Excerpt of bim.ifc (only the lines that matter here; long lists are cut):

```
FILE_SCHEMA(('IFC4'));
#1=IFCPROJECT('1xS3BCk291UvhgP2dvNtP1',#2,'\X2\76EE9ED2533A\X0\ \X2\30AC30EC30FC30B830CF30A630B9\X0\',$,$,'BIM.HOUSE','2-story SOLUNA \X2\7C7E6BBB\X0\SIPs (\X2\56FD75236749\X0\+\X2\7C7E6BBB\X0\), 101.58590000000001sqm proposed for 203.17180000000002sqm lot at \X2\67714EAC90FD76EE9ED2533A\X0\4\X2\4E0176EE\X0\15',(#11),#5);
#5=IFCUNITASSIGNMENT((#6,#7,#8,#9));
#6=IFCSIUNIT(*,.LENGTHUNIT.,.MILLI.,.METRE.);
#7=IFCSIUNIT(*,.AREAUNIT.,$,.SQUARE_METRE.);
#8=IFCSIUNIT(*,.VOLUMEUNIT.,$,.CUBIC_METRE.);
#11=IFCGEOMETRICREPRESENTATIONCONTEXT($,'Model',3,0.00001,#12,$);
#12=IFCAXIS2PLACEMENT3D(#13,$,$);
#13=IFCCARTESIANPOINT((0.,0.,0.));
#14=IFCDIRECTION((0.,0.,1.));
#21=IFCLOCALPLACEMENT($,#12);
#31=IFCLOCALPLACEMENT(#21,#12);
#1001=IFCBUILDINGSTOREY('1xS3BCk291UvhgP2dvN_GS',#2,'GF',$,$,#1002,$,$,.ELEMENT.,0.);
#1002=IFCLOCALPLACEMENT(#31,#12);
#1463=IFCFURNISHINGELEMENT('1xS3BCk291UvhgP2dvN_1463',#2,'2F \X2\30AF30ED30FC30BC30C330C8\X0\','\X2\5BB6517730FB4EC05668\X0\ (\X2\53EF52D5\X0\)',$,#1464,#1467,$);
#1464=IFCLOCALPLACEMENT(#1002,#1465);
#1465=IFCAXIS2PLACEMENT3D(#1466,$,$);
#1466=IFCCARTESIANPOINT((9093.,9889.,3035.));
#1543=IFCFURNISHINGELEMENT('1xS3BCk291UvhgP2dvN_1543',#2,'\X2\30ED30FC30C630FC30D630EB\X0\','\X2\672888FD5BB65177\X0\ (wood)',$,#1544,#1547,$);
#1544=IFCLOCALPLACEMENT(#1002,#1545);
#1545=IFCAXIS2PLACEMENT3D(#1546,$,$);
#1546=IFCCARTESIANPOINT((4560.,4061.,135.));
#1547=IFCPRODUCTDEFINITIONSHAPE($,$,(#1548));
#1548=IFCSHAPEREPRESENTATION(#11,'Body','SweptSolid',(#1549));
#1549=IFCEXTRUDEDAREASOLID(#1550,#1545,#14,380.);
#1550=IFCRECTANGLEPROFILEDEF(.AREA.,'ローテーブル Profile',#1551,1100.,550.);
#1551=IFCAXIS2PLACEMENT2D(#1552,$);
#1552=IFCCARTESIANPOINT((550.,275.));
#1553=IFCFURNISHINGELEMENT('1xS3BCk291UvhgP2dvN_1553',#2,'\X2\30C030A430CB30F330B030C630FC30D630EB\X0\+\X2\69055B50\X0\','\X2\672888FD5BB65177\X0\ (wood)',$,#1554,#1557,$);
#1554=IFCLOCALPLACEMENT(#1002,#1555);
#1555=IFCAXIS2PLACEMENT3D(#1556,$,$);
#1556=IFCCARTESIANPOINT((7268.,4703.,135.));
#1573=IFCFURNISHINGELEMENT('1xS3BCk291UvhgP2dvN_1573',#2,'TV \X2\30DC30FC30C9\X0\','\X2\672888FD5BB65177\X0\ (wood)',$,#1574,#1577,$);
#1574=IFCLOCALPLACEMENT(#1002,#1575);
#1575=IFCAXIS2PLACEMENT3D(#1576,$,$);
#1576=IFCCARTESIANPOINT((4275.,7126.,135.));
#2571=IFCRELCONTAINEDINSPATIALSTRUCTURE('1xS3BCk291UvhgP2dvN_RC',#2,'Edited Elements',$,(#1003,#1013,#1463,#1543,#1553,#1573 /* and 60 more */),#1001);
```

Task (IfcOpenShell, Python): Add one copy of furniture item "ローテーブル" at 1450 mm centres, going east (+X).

```python
import numpy as np
import ifcopenshell
import ifcopenshell.api.geometry
import ifcopenshell.api.root
import ifcopenshell.util.element
import ifcopenshell.util.placement

model = ifcopenshell.open("bim.ifc")


def reuse_history(source, copy):
    """copy_class also copies each property set's owner history, people and application; keep the originals."""
    for rel in copy.IsDefinedBy:
        if rel.is_a("IfcRelDefinesByProperties") and (history := rel.RelatingPropertyDefinition.OwnerHistory):
            rel.RelatingPropertyDefinition.OwnerHistory = source.OwnerHistory
            ifcopenshell.util.element.remove_deep2(model, history)


source = model.by_guid("1xS3BCk291UvhgP2dvN_1543")
base = ifcopenshell.util.placement.get_local_placement(source.ObjectPlacement)
step = np.array([1.0, 0.0, 0.0]) * 1450.0

for i in range(1, 2):
    copy = ifcopenshell.api.root.copy_class(model, product=source)
    copy.Representation = ifcopenshell.util.element.copy_deep(
        model, source.Representation, exclude=["IfcGeometricRepresentationContext", "IfcRepresentationMap"]
    )
    reuse_history(source, copy)
    matrix = base.copy()
    matrix[:3, 3] += i * step
    print("added at", matrix[:3, 3].round(3) + 0.0)
    ifcopenshell.api.geometry.edit_object_placement(model, product=copy, matrix=matrix, is_si=False)

model.write("bim-out.ifc")
```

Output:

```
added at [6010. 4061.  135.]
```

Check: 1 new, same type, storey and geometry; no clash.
